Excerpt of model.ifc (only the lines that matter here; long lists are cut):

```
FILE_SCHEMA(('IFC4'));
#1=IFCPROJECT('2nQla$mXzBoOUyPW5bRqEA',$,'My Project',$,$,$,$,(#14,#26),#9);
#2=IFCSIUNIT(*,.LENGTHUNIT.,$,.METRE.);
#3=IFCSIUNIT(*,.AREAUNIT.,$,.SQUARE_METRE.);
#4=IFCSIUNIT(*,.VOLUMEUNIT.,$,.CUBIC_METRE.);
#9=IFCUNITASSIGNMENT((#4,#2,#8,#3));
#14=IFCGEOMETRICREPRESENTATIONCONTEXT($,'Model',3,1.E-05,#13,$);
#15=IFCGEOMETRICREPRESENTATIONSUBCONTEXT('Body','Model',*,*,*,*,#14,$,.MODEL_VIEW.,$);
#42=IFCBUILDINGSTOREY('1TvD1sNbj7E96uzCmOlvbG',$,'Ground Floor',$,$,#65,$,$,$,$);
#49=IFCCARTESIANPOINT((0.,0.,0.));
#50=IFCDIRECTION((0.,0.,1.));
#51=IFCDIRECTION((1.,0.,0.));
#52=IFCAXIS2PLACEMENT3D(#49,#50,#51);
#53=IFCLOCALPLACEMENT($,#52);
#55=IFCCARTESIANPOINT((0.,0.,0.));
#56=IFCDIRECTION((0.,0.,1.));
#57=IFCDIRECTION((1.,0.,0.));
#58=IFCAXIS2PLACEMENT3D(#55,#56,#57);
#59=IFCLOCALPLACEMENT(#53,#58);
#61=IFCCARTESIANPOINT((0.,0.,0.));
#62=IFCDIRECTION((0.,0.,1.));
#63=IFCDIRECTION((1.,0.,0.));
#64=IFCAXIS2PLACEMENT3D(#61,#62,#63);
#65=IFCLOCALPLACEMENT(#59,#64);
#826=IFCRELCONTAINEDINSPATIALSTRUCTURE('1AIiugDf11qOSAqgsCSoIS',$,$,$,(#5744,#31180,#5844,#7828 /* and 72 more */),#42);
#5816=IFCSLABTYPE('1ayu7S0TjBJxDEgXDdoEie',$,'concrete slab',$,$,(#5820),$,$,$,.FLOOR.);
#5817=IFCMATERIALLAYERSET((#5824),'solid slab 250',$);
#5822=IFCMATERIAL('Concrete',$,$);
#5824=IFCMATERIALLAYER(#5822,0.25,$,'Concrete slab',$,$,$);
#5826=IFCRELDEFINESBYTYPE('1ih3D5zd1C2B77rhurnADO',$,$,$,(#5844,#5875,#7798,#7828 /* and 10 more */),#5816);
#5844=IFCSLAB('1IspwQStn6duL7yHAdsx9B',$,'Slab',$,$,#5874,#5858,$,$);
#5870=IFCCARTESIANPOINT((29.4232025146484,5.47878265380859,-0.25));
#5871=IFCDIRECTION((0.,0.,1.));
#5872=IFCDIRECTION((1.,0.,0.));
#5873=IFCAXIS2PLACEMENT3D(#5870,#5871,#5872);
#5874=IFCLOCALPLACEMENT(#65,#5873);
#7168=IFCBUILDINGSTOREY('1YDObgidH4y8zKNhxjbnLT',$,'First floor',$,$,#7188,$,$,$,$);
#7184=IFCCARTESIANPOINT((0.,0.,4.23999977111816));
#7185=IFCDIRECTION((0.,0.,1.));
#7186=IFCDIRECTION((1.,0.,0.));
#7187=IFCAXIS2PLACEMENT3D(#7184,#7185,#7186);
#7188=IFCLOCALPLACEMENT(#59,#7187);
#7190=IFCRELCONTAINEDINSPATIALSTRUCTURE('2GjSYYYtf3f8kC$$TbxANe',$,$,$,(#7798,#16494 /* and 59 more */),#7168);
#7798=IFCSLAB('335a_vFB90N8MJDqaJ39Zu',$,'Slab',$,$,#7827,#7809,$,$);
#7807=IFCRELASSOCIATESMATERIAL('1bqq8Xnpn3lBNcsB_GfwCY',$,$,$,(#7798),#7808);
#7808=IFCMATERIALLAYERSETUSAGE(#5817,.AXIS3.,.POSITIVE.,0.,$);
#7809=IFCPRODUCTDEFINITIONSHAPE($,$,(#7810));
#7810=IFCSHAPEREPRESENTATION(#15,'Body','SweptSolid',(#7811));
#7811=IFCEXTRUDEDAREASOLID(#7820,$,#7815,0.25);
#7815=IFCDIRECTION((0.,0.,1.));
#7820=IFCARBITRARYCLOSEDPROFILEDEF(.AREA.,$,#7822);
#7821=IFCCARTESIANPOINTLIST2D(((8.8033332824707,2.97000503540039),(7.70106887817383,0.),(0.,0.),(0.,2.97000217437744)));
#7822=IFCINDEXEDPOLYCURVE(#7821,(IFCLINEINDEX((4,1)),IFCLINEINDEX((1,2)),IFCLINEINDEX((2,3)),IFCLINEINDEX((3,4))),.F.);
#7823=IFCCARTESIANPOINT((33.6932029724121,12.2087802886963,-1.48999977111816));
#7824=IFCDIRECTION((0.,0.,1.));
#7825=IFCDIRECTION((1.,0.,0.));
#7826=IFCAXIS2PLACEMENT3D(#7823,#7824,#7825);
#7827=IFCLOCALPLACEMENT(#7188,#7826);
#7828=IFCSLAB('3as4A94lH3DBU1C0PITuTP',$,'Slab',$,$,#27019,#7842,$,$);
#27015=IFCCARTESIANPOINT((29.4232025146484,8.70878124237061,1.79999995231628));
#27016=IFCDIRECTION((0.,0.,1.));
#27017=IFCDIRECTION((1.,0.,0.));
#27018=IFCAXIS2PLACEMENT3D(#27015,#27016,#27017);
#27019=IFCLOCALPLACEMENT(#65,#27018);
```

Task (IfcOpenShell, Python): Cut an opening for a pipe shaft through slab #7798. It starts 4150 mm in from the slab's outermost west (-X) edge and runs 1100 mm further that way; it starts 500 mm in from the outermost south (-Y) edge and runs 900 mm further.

```python
import numpy as np
import ifcopenshell
import ifcopenshell.api.feature
import ifcopenshell.api.geometry
import ifcopenshell.api.root
import ifcopenshell.geom
import ifcopenshell.util.placement
import ifcopenshell.util.representation
import ifcopenshell.util.shape
import ifcopenshell.util.unit

model = ifcopenshell.open("model.ifc")
unit_scale = ifcopenshell.util.unit.calculate_unit_scale(model)
settings = ifcopenshell.geom.settings()


def volume(element):
    """Net volume in cubic metres, openings subtracted."""
    shape = ifcopenshell.geom.create_shape(settings, element)
    return ifcopenshell.util.shape.get_volume(shape.geometry)


slab = model.by_guid("335a_vFB90N8MJDqaJ39Zu")
before = volume(slab)

# Extent in the slab's own axes, in metres. The edges named are its -X and -Y sides.
slab_shape = ifcopenshell.geom.create_shape(settings, slab)
vertices = ifcopenshell.util.shape.get_vertices(slab_shape.geometry)
x_min, y_min, bottom = vertices.min(axis=0)
top = vertices[:, 2].max()

opening = ifcopenshell.api.root.create_entity(model, ifc_class="IfcOpeningElement", name="Pipe shaft opening", predefined_type="OPENING")
context = ifcopenshell.util.representation.get_context(model, "Model", "Body", "MODEL_VIEW")
width, depth = 1.1, 0.9
outline = [(0.0, 0.0), (width, 0.0), (width, depth), (0.0, depth), (0.0, 0.0)]
# Overshoot both faces by 50 mm so the cut is clean.
shape = ifcopenshell.api.geometry.add_slab_representation(
    model, context=context, depth=top - bottom + 0.1, polyline=outline
)
ifcopenshell.api.geometry.assign_representation(model, product=opening, representation=shape)

matrix = ifcopenshell.util.placement.get_local_placement(slab.ObjectPlacement)
matrix[:, 3] = matrix @ np.append(np.array([x_min + 4.15, y_min + 0.5, bottom - 0.05]) / unit_scale, 1.0)
ifcopenshell.api.geometry.edit_object_placement(model, product=opening, matrix=matrix, is_si=False)
ifcopenshell.api.feature.add_feature(model, feature=opening, element=slab)

after = volume(slab)

print(f"slab volume {before:.3f} -> {after:.3f} m3")

model.write("model_edited.ifc")
```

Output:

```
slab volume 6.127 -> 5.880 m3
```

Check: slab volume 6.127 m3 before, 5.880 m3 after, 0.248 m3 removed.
